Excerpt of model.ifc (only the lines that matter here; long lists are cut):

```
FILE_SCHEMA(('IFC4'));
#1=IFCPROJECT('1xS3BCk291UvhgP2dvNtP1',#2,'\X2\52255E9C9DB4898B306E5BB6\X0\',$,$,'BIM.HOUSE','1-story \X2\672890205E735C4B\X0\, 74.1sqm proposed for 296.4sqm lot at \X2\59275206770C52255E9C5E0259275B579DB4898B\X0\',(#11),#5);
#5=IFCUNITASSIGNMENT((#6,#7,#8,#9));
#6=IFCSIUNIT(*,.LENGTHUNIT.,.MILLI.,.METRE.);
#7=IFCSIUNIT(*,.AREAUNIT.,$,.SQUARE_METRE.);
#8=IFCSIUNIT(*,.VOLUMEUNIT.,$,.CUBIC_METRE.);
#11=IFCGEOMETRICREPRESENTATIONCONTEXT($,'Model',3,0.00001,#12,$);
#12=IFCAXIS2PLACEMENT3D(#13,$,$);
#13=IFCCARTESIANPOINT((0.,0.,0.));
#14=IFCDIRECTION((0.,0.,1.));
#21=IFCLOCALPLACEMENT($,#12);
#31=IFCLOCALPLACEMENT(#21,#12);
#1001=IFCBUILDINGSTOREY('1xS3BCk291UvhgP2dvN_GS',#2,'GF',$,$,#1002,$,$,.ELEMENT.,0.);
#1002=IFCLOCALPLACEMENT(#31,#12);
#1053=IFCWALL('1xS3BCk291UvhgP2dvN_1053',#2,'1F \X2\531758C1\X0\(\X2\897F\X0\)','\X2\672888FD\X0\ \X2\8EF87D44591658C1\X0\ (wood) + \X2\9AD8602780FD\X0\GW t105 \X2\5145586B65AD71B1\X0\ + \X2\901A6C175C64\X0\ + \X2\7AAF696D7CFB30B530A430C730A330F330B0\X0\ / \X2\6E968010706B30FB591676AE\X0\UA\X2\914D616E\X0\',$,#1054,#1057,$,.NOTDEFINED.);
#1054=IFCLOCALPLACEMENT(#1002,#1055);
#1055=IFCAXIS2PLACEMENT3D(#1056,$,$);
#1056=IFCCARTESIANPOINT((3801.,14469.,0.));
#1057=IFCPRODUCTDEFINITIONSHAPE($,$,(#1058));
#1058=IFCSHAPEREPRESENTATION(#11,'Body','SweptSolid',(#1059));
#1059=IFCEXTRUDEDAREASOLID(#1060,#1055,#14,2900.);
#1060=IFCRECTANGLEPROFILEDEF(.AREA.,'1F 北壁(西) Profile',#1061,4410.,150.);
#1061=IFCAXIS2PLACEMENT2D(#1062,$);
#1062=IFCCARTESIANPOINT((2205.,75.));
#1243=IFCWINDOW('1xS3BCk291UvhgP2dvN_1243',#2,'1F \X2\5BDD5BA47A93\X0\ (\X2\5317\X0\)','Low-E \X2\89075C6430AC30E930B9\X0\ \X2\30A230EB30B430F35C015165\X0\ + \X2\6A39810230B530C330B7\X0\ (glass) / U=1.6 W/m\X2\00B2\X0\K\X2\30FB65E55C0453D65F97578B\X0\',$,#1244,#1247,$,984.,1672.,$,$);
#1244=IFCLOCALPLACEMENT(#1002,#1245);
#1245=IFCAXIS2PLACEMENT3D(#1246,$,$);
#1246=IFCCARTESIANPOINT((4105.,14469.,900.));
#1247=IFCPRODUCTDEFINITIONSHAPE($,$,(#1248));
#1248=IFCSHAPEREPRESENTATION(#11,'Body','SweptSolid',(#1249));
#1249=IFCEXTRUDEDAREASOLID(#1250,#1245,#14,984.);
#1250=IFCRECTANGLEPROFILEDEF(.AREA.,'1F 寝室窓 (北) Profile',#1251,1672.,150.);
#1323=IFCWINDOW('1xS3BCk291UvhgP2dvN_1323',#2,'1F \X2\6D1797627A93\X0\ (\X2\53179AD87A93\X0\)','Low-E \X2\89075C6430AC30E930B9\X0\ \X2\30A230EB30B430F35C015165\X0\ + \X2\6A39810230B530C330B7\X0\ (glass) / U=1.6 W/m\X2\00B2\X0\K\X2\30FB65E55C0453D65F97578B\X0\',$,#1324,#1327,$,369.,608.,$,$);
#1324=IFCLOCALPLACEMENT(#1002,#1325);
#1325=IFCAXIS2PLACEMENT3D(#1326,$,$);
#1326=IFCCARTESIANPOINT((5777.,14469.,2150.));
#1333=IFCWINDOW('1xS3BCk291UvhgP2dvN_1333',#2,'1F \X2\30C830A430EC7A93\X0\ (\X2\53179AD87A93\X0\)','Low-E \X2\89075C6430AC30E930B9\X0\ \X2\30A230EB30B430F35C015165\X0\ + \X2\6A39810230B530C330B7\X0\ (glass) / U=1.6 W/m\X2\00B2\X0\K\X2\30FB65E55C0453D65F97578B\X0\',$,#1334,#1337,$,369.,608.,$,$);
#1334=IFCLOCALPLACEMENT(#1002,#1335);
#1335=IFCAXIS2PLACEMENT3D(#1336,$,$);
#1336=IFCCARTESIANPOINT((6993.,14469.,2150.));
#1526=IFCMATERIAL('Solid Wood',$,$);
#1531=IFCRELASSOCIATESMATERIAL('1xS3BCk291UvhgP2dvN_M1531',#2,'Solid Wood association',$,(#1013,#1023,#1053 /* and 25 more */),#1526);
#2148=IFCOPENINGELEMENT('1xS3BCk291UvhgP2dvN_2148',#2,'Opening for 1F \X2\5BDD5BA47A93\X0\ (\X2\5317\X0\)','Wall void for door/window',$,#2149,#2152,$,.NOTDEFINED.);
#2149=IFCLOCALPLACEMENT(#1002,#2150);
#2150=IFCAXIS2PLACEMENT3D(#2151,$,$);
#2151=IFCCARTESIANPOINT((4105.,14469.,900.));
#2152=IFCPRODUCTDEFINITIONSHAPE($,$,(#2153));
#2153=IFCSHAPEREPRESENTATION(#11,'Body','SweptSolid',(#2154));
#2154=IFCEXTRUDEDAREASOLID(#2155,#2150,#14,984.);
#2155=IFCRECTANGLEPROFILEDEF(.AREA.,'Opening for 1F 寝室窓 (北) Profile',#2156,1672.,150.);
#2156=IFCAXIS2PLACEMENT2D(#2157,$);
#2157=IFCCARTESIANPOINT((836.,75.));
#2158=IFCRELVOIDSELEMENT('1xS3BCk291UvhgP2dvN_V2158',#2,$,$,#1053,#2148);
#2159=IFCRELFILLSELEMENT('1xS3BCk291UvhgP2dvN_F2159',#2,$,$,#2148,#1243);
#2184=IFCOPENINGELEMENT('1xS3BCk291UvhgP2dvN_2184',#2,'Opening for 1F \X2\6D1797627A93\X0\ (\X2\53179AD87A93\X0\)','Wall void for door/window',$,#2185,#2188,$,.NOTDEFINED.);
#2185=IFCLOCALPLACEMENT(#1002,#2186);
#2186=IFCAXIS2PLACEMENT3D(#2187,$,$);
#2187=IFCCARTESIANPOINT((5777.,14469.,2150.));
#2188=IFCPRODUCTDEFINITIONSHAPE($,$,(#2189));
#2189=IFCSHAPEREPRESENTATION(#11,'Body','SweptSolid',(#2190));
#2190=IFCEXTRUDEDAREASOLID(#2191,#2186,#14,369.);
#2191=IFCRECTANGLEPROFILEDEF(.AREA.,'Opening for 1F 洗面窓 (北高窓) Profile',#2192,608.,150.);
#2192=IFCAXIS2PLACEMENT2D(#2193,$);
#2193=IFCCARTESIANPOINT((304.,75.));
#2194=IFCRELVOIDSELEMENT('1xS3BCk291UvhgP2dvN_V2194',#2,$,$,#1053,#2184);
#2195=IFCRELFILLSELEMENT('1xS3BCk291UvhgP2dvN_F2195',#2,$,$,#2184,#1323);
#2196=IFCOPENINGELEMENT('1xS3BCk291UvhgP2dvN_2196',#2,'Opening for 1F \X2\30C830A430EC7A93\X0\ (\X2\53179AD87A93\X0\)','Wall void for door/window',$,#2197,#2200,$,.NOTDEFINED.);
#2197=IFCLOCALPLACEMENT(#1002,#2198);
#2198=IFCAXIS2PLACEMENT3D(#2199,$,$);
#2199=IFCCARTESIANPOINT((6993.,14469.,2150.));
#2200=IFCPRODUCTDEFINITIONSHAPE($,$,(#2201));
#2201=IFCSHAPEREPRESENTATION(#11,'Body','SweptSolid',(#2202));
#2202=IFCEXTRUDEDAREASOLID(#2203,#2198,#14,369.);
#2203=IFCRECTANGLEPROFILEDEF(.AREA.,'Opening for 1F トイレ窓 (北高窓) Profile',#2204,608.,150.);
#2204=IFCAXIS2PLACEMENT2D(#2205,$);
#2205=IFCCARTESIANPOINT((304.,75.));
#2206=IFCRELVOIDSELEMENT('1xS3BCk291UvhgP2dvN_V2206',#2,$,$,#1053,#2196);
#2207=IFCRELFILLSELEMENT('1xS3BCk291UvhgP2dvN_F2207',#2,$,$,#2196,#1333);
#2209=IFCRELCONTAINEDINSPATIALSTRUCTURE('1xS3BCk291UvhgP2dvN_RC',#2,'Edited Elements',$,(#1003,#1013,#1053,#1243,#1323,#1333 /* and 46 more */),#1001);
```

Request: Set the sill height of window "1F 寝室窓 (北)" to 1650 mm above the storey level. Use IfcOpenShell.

```python
import numpy as np
import ifcopenshell
import ifcopenshell.api.geometry
import ifcopenshell.geom
import ifcopenshell.util.element
import ifcopenshell.util.placement
import ifcopenshell.util.shape
import ifcopenshell.util.unit

model = ifcopenshell.open("model.ifc")
unit_scale = ifcopenshell.util.unit.calculate_unit_scale(model)

window = model.by_guid("1xS3BCk291UvhgP2dvN_1243")
opening = window.FillsVoids[0].RelatingOpeningElement
storey = ifcopenshell.util.element.get_container(window, ifc_class="IfcBuildingStorey")
level = ifcopenshell.util.placement.get_local_placement(storey.ObjectPlacement)[2, 3]

# The opening's origin need not be at the sill, so measure its lowest point.
shape = ifcopenshell.geom.create_shape(ifcopenshell.geom.settings(), opening)
bottom = ifcopenshell.util.shape.get_shape_bottom_elevation(shape, shape.geometry) / unit_scale
dz = level + 1650.0 - bottom

shift = np.array([0.0, 0.0, dz])
# The window is not placed relative to its opening, so move both.
for product in (opening, window):
    matrix = ifcopenshell.util.placement.get_local_placement(product.ObjectPlacement)
    matrix[:3, 3] += shift
    ifcopenshell.api.geometry.edit_object_placement(model, product=product, matrix=matrix, is_si=False)

print(f"moved by {dz * unit_scale:+.3f} m")

model.write("model_updated.ifc")
```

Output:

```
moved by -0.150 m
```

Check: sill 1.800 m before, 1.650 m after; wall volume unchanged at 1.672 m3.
